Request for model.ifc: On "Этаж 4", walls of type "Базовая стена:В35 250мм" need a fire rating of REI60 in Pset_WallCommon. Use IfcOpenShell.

First a look at what the model holds.

```python
import ifcopenshell
import ifcopenshell.util.element

model = ifcopenshell.open("model.ifc")
print(model.schema)
storey = next(s for s in model.by_type("IfcBuildingStorey") if s.Name == "Этаж 4")
walls = [e for e in ifcopenshell.util.element.get_decomposition(storey) if e.is_a("IfcWall")]
seen = {}
for e in walls:
    element_type = ifcopenshell.util.element.get_type(e)
    key = (element_type.Name if element_type != e and element_type else None, ifcopenshell.util.element.get_pset(e, "Pset_WallCommon", "FireRating"))
    seen[key] = seen.get(key, 0) + 1
for (name, value), count in sorted(seen.items(), key=str):
    print(count, "x", name, "|", value)
```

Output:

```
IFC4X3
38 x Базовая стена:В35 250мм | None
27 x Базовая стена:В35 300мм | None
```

```python
import ifcopenshell
import ifcopenshell.api.pset
import ifcopenshell.util.element

model = ifcopenshell.open("model.ifc")

storey = next(s for s in model.by_type("IfcBuildingStorey") if s.Name == "Этаж 4")
walls = [e for e in ifcopenshell.util.element.get_decomposition(storey) if e.is_a("IfcWall")]

count = 0
for e in walls:
    element_type = ifcopenshell.util.element.get_type(e)
    if element_type in (None, e) or element_type.Name != "Базовая стена:В35 250мм":
        continue
    # add_pset returns the element's existing set when there is one.
    pset = ifcopenshell.api.pset.add_pset(model, product=e, name="Pset_WallCommon")
    ifcopenshell.api.pset.edit_pset(model, pset=pset, properties={"FireRating": "REI60"})
    count += 1

print(count, "walls updated")

model.write("model_v2.ifc")
```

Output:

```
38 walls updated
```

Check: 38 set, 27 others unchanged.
